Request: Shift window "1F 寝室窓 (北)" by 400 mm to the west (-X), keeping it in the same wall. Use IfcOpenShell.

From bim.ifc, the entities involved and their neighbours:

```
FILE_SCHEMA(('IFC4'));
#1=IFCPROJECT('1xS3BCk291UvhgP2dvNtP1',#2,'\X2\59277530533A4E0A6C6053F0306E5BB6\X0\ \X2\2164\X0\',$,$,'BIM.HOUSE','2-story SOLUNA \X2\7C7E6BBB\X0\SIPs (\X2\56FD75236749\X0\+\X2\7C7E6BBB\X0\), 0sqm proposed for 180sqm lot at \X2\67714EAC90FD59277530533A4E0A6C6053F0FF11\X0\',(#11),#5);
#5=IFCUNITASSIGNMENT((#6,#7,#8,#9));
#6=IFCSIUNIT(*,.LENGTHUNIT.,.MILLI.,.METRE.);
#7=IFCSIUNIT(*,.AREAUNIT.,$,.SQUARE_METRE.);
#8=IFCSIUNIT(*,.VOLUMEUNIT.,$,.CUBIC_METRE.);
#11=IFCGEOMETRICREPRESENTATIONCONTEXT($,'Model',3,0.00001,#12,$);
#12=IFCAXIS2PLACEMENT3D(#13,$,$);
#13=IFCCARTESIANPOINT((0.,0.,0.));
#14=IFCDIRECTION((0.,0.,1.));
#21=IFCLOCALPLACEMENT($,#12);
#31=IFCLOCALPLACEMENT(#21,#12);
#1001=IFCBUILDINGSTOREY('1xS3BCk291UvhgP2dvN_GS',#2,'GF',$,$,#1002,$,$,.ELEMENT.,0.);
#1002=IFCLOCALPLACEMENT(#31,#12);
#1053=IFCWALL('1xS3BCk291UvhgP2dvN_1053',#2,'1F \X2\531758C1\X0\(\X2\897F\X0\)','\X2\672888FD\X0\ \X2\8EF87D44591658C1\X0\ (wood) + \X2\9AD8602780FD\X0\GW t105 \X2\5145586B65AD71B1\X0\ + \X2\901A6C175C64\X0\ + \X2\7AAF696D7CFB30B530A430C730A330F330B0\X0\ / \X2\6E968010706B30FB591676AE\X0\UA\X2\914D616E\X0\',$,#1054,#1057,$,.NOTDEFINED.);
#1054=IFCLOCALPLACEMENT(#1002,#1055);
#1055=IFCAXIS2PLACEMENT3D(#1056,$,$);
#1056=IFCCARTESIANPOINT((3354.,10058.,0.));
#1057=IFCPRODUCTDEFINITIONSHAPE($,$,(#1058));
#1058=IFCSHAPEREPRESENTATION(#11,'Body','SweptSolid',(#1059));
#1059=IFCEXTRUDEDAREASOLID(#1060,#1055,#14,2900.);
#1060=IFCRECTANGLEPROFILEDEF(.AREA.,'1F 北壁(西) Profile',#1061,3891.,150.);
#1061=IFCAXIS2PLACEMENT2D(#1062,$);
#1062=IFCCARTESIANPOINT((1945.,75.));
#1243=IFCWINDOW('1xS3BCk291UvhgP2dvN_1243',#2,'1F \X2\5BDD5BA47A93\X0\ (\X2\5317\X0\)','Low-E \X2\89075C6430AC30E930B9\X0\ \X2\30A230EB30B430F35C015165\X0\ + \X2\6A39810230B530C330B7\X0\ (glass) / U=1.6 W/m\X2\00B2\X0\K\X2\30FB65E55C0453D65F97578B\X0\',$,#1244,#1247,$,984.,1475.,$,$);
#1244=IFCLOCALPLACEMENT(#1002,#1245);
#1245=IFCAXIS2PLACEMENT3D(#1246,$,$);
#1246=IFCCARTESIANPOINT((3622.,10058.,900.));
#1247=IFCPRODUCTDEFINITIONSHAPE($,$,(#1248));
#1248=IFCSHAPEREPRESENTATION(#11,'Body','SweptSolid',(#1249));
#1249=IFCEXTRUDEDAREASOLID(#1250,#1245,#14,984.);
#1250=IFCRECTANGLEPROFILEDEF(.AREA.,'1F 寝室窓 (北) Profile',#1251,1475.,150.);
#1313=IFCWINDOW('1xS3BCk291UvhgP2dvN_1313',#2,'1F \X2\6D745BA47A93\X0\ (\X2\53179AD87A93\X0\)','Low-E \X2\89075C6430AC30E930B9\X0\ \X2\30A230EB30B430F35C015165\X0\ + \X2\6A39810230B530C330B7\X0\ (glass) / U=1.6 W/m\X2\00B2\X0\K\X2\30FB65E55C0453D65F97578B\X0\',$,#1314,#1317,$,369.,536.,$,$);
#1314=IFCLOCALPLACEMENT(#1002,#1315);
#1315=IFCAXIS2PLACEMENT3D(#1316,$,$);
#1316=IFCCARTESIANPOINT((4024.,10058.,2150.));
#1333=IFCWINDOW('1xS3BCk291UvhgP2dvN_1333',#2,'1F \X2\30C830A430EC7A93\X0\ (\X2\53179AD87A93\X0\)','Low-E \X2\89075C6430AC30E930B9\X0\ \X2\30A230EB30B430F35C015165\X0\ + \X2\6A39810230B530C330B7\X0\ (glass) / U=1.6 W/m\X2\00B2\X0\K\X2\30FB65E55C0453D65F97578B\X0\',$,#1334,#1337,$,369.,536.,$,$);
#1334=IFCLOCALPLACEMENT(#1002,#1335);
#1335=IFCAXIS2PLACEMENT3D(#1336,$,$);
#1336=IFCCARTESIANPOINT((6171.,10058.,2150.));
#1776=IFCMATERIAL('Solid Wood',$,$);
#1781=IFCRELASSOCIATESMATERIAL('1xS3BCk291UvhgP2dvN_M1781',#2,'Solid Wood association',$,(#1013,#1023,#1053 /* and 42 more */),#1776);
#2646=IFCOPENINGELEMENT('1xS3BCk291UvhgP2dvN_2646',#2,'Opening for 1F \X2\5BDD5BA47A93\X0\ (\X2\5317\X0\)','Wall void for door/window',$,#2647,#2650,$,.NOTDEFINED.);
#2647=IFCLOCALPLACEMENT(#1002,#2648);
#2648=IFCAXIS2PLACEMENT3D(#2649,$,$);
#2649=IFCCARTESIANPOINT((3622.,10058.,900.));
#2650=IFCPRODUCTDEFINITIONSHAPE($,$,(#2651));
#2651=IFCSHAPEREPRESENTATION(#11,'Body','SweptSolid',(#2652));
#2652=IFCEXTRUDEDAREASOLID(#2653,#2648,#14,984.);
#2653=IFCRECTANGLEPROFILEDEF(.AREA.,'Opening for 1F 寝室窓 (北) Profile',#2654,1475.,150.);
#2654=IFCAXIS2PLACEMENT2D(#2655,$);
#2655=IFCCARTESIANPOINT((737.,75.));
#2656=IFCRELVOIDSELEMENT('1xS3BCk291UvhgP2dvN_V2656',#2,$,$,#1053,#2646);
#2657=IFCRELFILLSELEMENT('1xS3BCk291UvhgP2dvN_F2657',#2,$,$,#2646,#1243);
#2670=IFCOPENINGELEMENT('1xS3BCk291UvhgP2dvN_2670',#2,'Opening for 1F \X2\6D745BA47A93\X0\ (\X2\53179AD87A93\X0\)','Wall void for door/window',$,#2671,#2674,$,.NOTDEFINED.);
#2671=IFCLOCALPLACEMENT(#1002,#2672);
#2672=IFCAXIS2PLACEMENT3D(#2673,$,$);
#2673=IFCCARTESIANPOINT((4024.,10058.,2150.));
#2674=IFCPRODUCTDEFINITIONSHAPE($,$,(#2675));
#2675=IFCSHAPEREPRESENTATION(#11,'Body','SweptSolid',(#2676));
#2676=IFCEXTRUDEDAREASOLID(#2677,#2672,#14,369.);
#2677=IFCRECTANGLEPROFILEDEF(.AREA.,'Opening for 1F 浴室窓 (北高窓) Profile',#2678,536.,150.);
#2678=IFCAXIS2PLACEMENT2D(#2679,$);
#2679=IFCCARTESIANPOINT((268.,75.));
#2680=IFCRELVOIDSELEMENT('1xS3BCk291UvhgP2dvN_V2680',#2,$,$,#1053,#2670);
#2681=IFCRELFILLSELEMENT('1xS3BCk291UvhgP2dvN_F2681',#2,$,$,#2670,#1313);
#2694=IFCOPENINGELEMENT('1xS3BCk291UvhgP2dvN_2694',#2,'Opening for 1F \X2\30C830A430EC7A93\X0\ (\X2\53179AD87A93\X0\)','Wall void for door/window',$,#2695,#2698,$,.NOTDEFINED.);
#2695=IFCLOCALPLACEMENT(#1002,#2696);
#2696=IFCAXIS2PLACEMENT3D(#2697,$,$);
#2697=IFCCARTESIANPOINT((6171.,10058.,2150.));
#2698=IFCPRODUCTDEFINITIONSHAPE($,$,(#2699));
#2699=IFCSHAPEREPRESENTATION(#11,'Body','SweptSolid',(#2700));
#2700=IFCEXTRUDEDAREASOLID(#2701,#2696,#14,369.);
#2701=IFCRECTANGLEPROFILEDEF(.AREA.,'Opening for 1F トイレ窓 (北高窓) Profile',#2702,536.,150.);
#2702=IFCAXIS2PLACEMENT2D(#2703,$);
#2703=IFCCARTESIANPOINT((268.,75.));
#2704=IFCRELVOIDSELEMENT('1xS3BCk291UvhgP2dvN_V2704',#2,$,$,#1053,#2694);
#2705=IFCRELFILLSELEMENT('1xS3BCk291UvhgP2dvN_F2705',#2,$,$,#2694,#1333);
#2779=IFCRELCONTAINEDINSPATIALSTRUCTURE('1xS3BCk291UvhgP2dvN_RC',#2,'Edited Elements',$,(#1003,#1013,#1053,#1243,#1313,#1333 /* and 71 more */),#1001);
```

```python
import ifcopenshell
import ifcopenshell.api.geometry
import ifcopenshell.util.placement

model = ifcopenshell.open("bim.ifc")

window = model.by_guid("1xS3BCk291UvhgP2dvN_1243")
opening = window.FillsVoids[0].RelatingOpeningElement
wall = opening.VoidsElements[0].RelatingBuildingElement

wall_matrix = ifcopenshell.util.placement.get_local_placement(wall.ObjectPlacement)
shift = wall_matrix[:3, 0] * -400.0
before = ifcopenshell.util.placement.get_local_placement(window.ObjectPlacement)[:3, 3].copy()

# The window is not placed relative to its opening, so move both.
for product in (opening, window):
    matrix = ifcopenshell.util.placement.get_local_placement(product.ObjectPlacement)
    matrix[:3, 3] += shift
    ifcopenshell.api.geometry.edit_object_placement(model, product=product, matrix=matrix, is_si=False)

after = ifcopenshell.util.placement.get_local_placement(window.ObjectPlacement)[:3, 3]
print("window moved by", (after - before).round(3) + 0.0)

model.write("bim_updated.ifc")
```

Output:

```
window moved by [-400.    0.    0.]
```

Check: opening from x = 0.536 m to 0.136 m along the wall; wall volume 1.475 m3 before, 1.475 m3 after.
